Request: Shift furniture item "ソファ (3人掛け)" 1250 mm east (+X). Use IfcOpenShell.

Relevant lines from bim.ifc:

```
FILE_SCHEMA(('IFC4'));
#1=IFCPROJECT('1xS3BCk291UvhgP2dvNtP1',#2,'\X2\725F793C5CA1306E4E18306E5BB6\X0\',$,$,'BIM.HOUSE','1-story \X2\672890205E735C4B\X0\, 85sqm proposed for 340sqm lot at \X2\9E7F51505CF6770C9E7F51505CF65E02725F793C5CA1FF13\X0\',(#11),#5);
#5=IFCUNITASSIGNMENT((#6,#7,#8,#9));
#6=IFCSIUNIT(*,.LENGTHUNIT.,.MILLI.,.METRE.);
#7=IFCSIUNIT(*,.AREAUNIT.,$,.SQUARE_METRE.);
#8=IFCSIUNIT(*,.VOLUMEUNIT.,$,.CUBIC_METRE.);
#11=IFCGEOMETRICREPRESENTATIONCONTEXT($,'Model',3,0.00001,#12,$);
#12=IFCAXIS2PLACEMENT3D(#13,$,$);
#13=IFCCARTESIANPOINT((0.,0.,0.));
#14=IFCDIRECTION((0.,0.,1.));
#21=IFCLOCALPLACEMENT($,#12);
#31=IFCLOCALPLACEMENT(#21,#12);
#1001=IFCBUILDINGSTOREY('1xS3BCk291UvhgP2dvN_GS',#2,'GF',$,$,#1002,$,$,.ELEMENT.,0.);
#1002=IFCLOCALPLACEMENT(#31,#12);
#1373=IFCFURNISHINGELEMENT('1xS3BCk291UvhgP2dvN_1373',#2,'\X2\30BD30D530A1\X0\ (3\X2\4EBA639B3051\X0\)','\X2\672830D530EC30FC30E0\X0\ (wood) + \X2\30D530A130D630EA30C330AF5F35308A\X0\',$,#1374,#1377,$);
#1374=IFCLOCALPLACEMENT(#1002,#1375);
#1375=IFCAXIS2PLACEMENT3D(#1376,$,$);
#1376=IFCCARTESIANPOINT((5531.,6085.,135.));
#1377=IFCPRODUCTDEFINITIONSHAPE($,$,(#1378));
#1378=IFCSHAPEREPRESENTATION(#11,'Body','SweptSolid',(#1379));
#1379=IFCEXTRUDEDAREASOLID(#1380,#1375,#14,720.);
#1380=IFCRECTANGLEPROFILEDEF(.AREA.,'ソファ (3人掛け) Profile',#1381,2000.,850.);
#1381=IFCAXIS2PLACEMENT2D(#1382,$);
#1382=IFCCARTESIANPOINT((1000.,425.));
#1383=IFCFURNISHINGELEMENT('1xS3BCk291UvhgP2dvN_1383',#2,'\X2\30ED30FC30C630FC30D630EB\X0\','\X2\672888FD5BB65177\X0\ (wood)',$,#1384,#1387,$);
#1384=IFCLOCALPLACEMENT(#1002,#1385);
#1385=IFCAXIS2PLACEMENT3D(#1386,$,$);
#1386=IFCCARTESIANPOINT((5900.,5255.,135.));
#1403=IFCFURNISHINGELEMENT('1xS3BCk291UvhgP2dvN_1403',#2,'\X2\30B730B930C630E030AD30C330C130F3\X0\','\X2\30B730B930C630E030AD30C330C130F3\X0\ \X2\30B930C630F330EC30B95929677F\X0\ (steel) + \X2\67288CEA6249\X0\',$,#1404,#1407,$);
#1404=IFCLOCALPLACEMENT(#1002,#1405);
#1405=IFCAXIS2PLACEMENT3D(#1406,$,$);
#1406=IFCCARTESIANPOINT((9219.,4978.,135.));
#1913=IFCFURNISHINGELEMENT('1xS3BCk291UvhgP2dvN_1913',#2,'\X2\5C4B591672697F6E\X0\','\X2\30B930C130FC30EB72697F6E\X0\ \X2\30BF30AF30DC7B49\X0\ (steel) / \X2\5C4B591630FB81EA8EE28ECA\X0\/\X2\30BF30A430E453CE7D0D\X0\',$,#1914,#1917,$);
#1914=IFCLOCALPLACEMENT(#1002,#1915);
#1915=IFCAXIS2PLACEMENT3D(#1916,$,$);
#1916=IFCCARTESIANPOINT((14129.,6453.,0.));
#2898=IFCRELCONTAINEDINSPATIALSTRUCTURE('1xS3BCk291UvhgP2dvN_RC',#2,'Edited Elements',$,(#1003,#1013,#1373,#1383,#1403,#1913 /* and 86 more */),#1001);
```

```python
import ifcopenshell
import ifcopenshell.api.geometry
import ifcopenshell.util.placement
import ifcopenshell.util.unit

model = ifcopenshell.open("bim.ifc")
unit_scale = ifcopenshell.util.unit.calculate_unit_scale(model)

item = model.by_id(1373)
matrix = ifcopenshell.util.placement.get_local_placement(item.ObjectPlacement)
matrix[0, 3] += 1.25 / unit_scale
ifcopenshell.api.geometry.edit_object_placement(model, product=item, matrix=matrix, is_si=False)

print(ifcopenshell.util.placement.get_local_placement(item.ObjectPlacement).round(3) + 0.0)

model.write("bim-out.ifc")
```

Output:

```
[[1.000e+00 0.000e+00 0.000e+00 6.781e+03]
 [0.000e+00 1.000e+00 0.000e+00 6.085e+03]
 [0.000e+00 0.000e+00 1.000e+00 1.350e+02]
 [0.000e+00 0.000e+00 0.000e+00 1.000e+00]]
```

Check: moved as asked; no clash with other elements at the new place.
